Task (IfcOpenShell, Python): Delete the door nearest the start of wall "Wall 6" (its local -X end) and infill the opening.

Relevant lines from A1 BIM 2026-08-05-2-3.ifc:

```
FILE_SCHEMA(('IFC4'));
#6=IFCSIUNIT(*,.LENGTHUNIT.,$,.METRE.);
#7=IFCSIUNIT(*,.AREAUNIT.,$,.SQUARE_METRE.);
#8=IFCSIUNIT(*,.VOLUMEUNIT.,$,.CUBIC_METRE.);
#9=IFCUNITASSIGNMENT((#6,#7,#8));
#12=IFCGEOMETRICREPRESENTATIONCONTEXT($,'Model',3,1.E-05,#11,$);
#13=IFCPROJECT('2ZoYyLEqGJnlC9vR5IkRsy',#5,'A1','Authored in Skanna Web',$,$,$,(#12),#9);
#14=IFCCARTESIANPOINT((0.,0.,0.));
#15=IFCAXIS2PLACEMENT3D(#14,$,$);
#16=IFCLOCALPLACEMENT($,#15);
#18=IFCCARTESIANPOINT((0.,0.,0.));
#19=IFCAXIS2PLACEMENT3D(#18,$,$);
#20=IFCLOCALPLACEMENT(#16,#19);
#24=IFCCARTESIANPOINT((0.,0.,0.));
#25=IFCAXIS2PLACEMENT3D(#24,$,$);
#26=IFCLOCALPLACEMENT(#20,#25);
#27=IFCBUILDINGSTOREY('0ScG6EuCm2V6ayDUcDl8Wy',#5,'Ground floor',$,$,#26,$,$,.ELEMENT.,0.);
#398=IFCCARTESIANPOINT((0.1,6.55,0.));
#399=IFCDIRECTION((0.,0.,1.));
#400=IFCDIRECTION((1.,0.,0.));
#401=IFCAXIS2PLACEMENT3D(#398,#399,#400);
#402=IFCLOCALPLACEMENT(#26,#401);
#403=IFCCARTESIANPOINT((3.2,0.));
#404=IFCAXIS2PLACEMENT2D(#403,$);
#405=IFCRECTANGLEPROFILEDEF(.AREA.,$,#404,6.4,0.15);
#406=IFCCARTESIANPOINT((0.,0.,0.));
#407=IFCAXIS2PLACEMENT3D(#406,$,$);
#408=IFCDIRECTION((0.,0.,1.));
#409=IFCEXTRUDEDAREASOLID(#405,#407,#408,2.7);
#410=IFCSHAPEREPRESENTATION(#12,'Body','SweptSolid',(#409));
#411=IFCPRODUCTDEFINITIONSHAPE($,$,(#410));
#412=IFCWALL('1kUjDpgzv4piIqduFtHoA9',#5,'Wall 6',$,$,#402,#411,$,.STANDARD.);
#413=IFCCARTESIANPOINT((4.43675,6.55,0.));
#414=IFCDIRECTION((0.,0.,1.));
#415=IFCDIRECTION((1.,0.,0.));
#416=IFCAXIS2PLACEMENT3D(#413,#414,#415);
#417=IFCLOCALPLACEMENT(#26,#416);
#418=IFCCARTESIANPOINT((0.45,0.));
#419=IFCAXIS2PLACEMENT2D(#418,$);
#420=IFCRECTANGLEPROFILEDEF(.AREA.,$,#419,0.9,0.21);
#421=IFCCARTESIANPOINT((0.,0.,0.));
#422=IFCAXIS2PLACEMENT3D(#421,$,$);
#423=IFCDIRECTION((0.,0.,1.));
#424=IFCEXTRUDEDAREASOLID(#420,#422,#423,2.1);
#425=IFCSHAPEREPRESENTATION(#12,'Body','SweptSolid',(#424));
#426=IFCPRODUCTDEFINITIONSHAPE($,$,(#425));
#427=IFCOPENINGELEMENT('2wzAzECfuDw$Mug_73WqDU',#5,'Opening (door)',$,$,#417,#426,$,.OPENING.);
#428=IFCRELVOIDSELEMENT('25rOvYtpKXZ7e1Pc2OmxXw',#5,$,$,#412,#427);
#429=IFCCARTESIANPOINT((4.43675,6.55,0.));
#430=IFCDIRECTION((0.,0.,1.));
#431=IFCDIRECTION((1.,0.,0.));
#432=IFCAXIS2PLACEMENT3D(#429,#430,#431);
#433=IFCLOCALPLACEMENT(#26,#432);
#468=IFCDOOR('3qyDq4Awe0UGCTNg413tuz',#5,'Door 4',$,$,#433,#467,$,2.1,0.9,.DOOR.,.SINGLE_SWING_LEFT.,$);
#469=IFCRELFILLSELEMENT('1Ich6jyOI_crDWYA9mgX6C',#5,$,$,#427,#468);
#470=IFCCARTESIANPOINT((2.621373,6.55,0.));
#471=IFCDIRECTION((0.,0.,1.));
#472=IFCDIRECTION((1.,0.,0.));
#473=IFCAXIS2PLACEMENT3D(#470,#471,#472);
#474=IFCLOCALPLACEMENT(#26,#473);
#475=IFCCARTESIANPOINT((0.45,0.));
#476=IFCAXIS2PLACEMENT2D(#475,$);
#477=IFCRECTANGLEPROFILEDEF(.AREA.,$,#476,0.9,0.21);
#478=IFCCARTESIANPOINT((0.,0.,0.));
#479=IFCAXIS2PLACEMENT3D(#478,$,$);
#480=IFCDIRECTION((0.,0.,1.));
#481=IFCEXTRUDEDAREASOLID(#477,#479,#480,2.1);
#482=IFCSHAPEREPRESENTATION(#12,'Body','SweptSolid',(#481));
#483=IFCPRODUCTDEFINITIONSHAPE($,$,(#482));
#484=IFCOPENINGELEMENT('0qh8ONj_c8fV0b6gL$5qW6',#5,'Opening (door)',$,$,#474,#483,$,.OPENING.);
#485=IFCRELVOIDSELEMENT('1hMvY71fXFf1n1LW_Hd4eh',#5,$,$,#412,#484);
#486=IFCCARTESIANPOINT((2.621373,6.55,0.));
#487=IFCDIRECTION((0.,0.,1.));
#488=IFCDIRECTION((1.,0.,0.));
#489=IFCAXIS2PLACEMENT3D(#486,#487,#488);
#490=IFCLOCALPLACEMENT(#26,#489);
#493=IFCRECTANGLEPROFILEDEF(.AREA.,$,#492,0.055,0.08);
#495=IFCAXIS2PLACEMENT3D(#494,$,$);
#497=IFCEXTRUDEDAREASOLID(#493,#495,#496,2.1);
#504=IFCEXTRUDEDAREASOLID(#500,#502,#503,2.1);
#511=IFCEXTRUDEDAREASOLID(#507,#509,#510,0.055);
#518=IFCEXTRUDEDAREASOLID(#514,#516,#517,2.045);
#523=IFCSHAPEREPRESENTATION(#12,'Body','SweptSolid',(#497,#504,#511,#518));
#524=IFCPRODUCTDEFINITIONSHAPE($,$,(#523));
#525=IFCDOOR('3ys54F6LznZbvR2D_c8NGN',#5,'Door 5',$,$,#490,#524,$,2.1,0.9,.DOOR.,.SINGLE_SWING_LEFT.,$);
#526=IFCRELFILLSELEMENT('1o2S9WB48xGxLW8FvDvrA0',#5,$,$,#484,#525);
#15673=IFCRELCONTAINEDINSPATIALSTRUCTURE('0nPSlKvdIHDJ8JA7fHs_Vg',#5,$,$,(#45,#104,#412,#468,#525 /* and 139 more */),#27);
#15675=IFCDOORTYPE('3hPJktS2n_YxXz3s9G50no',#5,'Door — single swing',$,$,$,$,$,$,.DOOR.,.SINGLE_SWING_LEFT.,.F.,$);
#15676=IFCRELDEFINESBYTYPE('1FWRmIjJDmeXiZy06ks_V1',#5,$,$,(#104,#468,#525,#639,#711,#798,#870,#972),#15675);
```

```python
import ifcopenshell
import ifcopenshell.api.feature
import ifcopenshell.api.root
import ifcopenshell.geom
import ifcopenshell.util.shape

model = ifcopenshell.open("A1 BIM 2026-08-05-2-3.ifc")
settings = ifcopenshell.geom.settings()


def volume(element):
    """Net volume in cubic metres, openings subtracted."""
    shape = ifcopenshell.geom.create_shape(settings, element)
    return ifcopenshell.util.shape.get_volume(shape.geometry)


door = model.by_guid("3ys54F6LznZbvR2D_c8NGN")
opening = door.FillsVoids[0].RelatingOpeningElement
wall = opening.VoidsElements[0].RelatingBuildingElement
before = volume(wall)

ifcopenshell.api.root.remove_product(model, product=door)
ifcopenshell.api.feature.remove_feature(model, feature=opening)

after = volume(wall)

print(f"wall volume {before:.3f} -> {after:.3f} m3")

model.write("A1 BIM 2026-08-05-2-3_edited.ifc")
```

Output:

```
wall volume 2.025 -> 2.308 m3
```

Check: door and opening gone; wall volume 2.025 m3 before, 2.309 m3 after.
